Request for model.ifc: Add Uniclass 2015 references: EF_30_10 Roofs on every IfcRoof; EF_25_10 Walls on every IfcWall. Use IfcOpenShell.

First a look at what the model holds.

```python
import ifcopenshell

model = ifcopenshell.open("model.ifc")
print(model.schema)
print("classifications:", [c.Name for c in model.by_type("IfcClassification")])
for ifc_class in ("IfcDoor", "IfcRoof", "IfcStair", "IfcWall", "IfcWindow"):
    print(ifc_class, len(model.by_type(ifc_class)))
```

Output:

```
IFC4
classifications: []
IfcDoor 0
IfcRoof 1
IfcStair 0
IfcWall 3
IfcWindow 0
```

```python
import ifcopenshell
import ifcopenshell.api.classification

model = ifcopenshell.open("model.ifc")

system = ifcopenshell.api.classification.add_classification(model, classification="Uniclass 2015")

codes = {
    "IfcRoof": ("EF_30_10", "Roofs"),
    "IfcWall": ("EF_25_10", "Walls"),
}
for ifc_class, (code, name) in codes.items():
    products = model.by_type(ifc_class)
    ifcopenshell.api.classification.add_reference(
        model, products=products, classification=system, identification=code, name=name
    )
    print(code, len(products))

model.write("model_updated.ifc")
```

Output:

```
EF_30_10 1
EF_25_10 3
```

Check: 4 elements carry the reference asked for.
